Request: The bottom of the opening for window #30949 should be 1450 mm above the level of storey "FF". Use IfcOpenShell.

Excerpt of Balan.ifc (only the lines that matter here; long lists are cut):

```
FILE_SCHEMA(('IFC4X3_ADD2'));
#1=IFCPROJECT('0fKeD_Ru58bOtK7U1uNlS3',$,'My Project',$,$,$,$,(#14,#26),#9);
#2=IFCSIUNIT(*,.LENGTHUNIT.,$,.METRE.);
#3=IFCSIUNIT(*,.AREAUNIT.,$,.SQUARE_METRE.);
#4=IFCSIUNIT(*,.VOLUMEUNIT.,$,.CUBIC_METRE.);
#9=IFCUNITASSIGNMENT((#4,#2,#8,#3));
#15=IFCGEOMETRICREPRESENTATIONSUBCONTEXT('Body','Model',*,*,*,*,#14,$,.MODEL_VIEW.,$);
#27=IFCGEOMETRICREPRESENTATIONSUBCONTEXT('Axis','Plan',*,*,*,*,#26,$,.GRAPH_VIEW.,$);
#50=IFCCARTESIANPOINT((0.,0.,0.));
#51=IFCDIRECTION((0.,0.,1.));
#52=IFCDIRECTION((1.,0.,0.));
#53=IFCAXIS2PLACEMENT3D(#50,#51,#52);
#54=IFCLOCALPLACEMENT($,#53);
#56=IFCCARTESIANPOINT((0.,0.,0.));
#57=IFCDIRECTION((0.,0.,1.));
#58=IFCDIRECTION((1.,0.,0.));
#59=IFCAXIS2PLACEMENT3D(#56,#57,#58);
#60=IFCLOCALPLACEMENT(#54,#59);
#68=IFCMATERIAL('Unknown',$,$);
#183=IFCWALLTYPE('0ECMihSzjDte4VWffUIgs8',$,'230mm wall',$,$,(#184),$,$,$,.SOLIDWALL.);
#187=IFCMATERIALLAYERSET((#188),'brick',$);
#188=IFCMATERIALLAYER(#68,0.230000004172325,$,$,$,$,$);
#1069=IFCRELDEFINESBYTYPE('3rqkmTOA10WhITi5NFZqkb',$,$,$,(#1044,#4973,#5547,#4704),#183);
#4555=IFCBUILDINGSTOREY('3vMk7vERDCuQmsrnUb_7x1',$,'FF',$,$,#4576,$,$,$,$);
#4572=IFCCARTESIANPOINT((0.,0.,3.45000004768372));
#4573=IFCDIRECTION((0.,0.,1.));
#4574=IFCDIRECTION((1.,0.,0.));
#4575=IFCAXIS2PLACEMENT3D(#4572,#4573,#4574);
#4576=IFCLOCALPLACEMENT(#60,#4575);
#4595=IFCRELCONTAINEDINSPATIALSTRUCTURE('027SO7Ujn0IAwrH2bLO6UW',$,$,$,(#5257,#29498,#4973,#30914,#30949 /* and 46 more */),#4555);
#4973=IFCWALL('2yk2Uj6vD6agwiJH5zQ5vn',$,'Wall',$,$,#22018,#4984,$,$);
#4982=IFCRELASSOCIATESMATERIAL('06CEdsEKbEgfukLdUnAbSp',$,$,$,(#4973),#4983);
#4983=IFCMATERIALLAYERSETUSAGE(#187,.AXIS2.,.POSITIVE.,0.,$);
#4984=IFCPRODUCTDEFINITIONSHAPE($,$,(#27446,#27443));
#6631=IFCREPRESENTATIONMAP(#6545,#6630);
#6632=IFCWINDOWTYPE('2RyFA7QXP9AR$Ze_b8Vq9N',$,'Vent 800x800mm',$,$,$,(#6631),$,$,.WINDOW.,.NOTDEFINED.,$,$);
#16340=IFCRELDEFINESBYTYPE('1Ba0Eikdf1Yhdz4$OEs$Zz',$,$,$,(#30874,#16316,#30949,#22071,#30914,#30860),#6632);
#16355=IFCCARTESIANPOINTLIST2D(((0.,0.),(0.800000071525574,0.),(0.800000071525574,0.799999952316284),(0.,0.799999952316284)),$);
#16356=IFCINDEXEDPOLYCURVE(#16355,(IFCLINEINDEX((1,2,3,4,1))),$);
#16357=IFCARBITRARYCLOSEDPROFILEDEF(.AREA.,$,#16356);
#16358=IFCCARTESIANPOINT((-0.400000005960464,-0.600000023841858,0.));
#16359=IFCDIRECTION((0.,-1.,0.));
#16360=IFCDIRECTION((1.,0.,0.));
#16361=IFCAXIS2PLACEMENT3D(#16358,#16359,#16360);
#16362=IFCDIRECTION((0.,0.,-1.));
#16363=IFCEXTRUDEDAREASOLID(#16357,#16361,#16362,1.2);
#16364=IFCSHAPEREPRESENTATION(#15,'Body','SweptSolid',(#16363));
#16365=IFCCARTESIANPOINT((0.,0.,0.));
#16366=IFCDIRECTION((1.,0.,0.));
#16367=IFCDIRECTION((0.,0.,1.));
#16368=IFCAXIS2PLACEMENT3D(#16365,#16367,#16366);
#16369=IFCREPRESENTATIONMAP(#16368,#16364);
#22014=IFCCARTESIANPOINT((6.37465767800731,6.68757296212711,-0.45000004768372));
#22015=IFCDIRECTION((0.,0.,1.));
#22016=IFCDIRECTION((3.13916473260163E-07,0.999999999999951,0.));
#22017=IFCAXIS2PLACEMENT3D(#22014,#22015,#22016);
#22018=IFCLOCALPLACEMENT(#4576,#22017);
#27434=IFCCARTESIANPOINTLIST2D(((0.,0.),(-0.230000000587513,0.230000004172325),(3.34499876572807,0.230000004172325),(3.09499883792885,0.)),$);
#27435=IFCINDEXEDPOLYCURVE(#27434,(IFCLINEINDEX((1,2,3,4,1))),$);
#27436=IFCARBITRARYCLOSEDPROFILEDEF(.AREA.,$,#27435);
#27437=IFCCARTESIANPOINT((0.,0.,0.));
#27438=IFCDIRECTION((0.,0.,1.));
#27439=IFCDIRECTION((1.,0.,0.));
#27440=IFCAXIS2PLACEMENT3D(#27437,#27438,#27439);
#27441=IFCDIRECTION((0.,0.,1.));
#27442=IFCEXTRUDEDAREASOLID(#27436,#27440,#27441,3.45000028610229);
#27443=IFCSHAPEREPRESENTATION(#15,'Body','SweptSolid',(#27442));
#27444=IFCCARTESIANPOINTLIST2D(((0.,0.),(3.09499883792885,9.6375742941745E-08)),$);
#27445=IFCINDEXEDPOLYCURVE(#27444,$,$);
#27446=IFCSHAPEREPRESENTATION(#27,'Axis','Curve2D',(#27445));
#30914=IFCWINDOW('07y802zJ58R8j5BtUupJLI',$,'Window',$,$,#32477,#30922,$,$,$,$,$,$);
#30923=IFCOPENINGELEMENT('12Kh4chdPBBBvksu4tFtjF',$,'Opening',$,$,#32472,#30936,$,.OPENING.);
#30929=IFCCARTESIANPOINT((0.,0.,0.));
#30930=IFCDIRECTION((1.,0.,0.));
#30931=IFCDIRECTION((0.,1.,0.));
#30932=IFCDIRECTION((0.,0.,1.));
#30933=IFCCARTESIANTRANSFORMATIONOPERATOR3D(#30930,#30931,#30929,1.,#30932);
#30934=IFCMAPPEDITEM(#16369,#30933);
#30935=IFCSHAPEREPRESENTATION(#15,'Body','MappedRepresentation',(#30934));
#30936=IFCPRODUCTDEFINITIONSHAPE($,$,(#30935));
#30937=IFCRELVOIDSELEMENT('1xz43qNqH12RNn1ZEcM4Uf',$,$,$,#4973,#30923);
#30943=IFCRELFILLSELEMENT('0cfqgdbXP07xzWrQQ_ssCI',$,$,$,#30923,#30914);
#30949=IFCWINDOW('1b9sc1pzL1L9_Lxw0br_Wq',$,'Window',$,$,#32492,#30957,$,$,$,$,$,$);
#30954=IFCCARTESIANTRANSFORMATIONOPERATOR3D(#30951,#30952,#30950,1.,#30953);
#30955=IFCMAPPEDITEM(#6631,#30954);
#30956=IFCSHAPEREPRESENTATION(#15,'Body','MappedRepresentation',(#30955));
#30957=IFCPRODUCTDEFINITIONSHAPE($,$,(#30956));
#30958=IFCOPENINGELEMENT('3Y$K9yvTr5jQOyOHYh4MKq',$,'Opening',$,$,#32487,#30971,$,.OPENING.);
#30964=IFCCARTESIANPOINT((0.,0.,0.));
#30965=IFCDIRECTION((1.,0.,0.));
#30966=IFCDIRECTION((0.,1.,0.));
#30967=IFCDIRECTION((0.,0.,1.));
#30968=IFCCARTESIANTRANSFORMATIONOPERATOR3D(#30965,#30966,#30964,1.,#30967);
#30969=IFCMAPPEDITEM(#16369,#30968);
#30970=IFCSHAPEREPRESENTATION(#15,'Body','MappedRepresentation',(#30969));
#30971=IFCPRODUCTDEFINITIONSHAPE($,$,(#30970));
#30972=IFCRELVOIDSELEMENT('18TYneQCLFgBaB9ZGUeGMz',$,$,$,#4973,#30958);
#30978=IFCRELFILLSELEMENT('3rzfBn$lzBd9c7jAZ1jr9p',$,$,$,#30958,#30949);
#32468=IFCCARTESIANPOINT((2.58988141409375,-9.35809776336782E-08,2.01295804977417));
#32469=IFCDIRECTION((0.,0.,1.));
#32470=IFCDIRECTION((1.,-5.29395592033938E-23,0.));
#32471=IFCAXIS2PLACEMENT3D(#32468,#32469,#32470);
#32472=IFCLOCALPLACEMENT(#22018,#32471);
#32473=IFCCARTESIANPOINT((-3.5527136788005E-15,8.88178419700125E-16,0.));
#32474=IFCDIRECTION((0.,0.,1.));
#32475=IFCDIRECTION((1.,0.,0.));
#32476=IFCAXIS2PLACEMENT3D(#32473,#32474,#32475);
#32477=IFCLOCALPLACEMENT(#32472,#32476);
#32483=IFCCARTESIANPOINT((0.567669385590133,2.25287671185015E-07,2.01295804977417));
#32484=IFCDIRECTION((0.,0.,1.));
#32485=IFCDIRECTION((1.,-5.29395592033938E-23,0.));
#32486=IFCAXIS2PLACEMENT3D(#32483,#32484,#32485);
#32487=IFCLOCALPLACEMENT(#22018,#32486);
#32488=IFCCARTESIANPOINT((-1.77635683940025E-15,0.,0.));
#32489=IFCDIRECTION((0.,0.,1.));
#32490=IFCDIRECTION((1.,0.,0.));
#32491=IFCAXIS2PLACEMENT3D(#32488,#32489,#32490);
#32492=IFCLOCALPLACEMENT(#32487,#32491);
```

```python
import numpy as np
import ifcopenshell
import ifcopenshell.api.geometry
import ifcopenshell.geom
import ifcopenshell.util.element
import ifcopenshell.util.placement
import ifcopenshell.util.shape
import ifcopenshell.util.unit

model = ifcopenshell.open("Balan.ifc")
unit_scale = ifcopenshell.util.unit.calculate_unit_scale(model)

window = model.by_guid("1b9sc1pzL1L9_Lxw0br_Wq")
opening = window.FillsVoids[0].RelatingOpeningElement
storey = ifcopenshell.util.element.get_container(window, ifc_class="IfcBuildingStorey")
level = ifcopenshell.util.placement.get_local_placement(storey.ObjectPlacement)[2, 3]

# The opening's origin need not be at the sill, so measure its lowest point.
shape = ifcopenshell.geom.create_shape(ifcopenshell.geom.settings(), opening)
bottom = ifcopenshell.util.shape.get_shape_bottom_elevation(shape, shape.geometry) / unit_scale
dz = level + 1.45 - bottom

shift = np.array([0.0, 0.0, dz])
# The window is placed relative to its opening, so it follows when the opening moves.
matrix = ifcopenshell.util.placement.get_local_placement(opening.ObjectPlacement)
matrix[:3, 3] += shift
ifcopenshell.api.geometry.edit_object_placement(
    model, product=opening, matrix=matrix, is_si=False, should_transform_children=True
)

print(f"moved by {dz * unit_scale:+.3f} m")

model.write("Balan_updated.ifc")
```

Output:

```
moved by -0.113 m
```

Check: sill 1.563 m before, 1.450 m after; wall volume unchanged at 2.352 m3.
